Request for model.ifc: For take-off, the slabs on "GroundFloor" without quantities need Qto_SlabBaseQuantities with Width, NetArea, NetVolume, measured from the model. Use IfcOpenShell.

First a look at what the model holds.

```python
import ifcopenshell
import ifcopenshell.util.element
import ifcopenshell.util.unit

model = ifcopenshell.open("model.ifc")
print(model.schema)
for unit_type in ("LENGTHUNIT", "AREAUNIT", "VOLUMEUNIT"):
    print(unit_type, ifcopenshell.util.unit.calculate_unit_scale(model, unit_type))
storey = next(s for s in model.by_type("IfcBuildingStorey") if s.Name == "GroundFloor")
slabs = [e for e in ifcopenshell.util.element.get_decomposition(storey) if e.is_a("IfcSlab")]
for e in sorted(slabs, key=lambda e: e.id()):
    print(e.id(), e.is_a(), e.Name, list(ifcopenshell.util.element.get_psets(e, qtos_only=True)), sep=" | ")
```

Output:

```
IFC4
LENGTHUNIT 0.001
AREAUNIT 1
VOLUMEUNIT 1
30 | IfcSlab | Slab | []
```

```python
import ifcopenshell
import ifcopenshell.api.pset
import ifcopenshell.geom
import ifcopenshell.util.element
import ifcopenshell.util.shape
import ifcopenshell.util.unit

model = ifcopenshell.open("model.ifc")
unit_scale = ifcopenshell.util.unit.calculate_unit_scale(model)
area_scale = ifcopenshell.util.unit.calculate_unit_scale(model, "AREAUNIT")
volume_scale = ifcopenshell.util.unit.calculate_unit_scale(model, "VOLUMEUNIT")
settings = ifcopenshell.geom.settings()

storey = next(s for s in model.by_type("IfcBuildingStorey") if s.Name == "GroundFloor")
slabs = [e for e in ifcopenshell.util.element.get_decomposition(storey) if e.is_a("IfcSlab")]

for e in sorted(slabs, key=lambda e: e.id()):
    if ifcopenshell.util.element.get_psets(e, qtos_only=True, should_inherit=False):
        continue
    # Geometry comes back in metres, in the element's own axes.
    shape = ifcopenshell.geom.create_shape(settings, e)
    values = {
        "Width": ifcopenshell.util.shape.get_z(shape.geometry) / unit_scale,
        "NetArea": ifcopenshell.util.shape.get_footprint_area(shape.geometry) / area_scale,
        "NetVolume": ifcopenshell.util.shape.get_volume(shape.geometry) / volume_scale,
    }
    qto = ifcopenshell.api.pset.add_qto(model, product=e, name="Qto_SlabBaseQuantities")
    ifcopenshell.api.pset.edit_qto(model, qto=qto, properties=values)
    print(e.id(), {k: round(v, 3) for k, v in values.items()})

model.write("model-out.ifc")
```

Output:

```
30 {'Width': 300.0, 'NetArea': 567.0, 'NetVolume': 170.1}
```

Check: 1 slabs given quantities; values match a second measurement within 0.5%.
